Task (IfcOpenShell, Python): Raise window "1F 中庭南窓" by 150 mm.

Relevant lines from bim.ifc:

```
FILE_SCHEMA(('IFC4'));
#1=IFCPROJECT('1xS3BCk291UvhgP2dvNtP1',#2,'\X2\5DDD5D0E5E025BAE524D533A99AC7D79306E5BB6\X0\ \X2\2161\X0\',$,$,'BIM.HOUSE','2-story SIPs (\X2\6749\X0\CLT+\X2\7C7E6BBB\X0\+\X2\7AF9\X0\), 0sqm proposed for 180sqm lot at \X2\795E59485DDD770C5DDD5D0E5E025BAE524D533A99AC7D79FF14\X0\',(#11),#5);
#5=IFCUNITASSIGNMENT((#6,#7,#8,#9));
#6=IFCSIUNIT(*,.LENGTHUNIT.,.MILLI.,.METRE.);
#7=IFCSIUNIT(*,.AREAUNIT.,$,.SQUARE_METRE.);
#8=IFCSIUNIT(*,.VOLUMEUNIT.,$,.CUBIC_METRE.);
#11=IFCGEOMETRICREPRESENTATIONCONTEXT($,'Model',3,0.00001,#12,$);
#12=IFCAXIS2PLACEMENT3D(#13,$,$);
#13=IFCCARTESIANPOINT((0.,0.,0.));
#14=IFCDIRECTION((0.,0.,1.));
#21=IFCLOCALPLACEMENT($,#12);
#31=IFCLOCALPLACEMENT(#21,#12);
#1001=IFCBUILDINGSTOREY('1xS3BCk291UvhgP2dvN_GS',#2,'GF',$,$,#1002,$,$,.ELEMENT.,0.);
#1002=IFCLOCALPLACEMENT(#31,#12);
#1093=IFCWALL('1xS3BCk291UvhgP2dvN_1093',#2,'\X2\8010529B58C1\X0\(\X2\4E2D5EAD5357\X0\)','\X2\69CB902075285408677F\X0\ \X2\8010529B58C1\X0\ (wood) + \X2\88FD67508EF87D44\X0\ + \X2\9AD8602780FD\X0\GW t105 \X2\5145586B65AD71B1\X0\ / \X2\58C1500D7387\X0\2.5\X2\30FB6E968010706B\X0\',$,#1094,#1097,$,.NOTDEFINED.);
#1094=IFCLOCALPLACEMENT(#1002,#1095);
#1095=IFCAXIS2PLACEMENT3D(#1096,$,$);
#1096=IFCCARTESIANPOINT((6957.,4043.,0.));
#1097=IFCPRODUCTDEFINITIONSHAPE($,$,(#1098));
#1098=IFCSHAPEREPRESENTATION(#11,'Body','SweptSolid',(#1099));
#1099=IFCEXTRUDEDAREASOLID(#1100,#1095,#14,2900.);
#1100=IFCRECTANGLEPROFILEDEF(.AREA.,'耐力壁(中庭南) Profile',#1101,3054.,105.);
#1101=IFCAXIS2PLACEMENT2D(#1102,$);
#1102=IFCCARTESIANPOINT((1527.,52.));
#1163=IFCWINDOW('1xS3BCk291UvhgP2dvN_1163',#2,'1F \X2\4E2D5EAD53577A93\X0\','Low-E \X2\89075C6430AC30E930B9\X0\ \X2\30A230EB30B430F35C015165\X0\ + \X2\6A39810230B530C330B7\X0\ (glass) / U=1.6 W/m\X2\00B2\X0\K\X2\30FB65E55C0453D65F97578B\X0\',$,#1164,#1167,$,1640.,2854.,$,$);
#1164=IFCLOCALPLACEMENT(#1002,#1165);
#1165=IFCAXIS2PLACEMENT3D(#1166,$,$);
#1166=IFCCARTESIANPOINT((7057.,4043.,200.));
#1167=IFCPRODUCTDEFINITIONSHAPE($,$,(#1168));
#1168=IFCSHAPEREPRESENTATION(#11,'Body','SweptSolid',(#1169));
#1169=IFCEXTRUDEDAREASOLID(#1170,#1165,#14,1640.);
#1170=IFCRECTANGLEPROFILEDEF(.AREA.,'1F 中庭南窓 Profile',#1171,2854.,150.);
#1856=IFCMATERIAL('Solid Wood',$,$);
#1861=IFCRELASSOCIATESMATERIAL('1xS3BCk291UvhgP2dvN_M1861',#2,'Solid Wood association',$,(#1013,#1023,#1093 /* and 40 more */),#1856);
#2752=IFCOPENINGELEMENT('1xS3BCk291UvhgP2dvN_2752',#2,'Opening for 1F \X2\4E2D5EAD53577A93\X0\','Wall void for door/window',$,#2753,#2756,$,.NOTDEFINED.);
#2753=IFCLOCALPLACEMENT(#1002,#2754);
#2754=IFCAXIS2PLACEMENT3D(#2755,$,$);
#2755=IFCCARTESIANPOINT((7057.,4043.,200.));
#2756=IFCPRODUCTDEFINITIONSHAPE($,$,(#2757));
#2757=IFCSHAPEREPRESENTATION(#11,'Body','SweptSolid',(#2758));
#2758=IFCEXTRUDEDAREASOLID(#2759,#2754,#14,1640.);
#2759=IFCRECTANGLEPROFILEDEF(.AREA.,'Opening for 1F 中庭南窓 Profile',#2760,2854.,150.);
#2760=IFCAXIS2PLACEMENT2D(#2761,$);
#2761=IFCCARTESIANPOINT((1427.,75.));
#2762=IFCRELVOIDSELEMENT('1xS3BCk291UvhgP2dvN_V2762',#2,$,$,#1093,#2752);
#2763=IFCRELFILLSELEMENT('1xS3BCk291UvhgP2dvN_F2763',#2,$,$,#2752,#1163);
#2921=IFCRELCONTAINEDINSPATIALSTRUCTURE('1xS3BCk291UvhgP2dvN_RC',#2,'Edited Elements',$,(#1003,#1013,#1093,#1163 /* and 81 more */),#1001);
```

```python
import numpy as np
import ifcopenshell
import ifcopenshell.api.geometry
import ifcopenshell.util.placement
import ifcopenshell.util.unit

model = ifcopenshell.open("bim.ifc")
unit_scale = ifcopenshell.util.unit.calculate_unit_scale(model)

window = model.by_id(1163)
opening = window.FillsVoids[0].RelatingOpeningElement
dz = 0.15 / unit_scale

shift = np.array([0.0, 0.0, dz])
# The window is not placed relative to its opening, so move both.
for product in (opening, window):
    matrix = ifcopenshell.util.placement.get_local_placement(product.ObjectPlacement)
    matrix[:3, 3] += shift
    ifcopenshell.api.geometry.edit_object_placement(model, product=product, matrix=matrix, is_si=False)

print(f"moved by {dz * unit_scale:+.3f} m")

model.write("bim-out.ifc")
```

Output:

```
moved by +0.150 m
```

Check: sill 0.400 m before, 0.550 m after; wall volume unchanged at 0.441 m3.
